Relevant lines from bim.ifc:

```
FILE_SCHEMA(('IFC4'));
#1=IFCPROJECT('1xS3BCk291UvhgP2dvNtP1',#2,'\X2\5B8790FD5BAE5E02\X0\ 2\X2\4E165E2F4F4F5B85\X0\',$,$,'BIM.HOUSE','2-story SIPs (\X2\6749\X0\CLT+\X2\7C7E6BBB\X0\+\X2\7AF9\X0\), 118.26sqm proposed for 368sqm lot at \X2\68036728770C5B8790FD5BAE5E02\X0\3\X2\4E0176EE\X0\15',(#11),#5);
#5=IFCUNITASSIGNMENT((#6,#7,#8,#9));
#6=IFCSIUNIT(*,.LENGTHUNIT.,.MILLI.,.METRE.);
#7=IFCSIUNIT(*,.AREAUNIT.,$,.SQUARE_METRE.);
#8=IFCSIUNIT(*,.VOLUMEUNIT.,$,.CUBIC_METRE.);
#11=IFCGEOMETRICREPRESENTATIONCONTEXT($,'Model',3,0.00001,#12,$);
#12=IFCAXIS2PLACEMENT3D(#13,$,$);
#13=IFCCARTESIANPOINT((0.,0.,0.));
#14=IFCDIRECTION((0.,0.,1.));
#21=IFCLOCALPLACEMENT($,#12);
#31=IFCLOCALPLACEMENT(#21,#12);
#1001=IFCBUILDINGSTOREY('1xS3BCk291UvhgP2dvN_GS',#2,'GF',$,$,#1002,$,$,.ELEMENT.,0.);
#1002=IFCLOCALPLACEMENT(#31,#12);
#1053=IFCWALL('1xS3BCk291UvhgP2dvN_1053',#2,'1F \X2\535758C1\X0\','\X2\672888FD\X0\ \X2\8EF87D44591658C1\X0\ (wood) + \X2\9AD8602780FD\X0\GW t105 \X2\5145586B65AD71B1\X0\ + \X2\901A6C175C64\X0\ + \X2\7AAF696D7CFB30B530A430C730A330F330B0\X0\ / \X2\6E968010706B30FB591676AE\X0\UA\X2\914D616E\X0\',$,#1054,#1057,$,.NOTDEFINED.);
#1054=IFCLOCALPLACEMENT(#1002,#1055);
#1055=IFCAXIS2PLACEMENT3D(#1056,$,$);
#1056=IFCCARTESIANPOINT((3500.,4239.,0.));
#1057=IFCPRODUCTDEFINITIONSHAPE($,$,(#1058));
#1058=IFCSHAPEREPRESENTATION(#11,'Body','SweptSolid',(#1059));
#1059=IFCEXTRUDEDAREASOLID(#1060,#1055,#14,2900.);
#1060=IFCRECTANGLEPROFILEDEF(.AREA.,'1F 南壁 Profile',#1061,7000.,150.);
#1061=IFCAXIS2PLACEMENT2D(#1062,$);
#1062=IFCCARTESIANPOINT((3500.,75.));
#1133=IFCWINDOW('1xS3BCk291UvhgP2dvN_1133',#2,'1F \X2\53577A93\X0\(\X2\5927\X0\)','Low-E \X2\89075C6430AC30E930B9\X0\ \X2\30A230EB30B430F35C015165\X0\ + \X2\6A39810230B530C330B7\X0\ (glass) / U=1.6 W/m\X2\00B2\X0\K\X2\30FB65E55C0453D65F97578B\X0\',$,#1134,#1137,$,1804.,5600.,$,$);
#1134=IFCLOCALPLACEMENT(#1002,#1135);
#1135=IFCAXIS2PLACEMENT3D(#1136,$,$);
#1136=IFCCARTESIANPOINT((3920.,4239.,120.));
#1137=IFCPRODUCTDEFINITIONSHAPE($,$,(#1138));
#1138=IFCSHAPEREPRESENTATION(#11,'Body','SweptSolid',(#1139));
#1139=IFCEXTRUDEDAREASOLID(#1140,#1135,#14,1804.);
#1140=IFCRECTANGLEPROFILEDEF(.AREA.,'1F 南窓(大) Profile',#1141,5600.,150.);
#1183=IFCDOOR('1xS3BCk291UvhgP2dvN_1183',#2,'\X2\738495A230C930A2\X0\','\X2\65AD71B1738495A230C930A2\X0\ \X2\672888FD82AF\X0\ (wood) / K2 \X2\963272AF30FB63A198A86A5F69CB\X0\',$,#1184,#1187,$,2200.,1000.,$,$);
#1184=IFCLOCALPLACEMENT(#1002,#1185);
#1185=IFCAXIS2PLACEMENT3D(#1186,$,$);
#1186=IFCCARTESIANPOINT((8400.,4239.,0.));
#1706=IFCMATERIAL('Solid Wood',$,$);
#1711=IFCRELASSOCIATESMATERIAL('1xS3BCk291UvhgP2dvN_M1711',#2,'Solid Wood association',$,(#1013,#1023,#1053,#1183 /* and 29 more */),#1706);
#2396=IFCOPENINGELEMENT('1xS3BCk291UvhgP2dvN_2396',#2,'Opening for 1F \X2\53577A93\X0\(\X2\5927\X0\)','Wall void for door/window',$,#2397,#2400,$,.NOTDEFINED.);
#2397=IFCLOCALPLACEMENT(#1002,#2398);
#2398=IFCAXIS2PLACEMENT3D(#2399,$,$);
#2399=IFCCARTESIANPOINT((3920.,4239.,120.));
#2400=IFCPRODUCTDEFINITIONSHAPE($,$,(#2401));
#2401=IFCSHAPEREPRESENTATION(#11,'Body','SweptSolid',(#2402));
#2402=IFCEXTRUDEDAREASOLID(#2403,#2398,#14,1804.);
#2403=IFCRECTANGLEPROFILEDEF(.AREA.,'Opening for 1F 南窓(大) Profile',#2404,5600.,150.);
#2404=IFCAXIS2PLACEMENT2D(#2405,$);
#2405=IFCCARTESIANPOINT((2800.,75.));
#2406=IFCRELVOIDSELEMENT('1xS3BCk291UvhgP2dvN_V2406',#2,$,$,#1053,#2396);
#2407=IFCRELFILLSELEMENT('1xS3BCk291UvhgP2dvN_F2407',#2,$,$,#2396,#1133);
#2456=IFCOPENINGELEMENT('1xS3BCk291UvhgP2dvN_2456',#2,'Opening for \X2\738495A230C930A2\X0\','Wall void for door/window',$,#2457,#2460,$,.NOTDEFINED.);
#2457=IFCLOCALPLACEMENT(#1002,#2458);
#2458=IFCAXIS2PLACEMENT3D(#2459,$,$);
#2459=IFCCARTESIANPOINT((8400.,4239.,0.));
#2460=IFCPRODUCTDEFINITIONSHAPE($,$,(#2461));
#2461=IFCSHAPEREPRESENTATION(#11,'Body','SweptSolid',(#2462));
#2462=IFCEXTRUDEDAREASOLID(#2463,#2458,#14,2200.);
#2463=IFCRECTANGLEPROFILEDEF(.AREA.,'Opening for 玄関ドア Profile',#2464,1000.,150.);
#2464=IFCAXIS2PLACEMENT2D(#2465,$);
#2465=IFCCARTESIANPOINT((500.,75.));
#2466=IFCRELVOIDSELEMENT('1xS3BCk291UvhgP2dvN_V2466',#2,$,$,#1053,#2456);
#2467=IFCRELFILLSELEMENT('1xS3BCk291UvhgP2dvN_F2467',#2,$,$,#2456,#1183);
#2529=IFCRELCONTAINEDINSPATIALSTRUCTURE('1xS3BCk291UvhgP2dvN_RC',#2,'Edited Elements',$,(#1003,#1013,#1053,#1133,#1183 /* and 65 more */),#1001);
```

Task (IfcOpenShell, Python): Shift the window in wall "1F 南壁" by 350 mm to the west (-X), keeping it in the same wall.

```python
import ifcopenshell
import ifcopenshell.api.geometry
import ifcopenshell.util.placement
import ifcopenshell.util.unit

model = ifcopenshell.open("bim.ifc")
unit_scale = ifcopenshell.util.unit.calculate_unit_scale(model)

window = model.by_id(1133)
opening = window.FillsVoids[0].RelatingOpeningElement
wall = opening.VoidsElements[0].RelatingBuildingElement

wall_matrix = ifcopenshell.util.placement.get_local_placement(wall.ObjectPlacement)
shift = wall_matrix[:3, 0] * -0.35 / unit_scale
before = ifcopenshell.util.placement.get_local_placement(window.ObjectPlacement)[:3, 3].copy()

# The window is not placed relative to its opening, so move both.
for product in (opening, window):
    matrix = ifcopenshell.util.placement.get_local_placement(product.ObjectPlacement)
    matrix[:3, 3] += shift
    ifcopenshell.api.geometry.edit_object_placement(model, product=product, matrix=matrix, is_si=False)

after = ifcopenshell.util.placement.get_local_placement(window.ObjectPlacement)[:3, 3]
print("window moved by", (after - before).round(3) + 0.0)

model.write("bim-out.ifc")
```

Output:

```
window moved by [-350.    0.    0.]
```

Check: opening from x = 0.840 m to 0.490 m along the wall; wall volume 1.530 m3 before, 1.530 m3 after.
